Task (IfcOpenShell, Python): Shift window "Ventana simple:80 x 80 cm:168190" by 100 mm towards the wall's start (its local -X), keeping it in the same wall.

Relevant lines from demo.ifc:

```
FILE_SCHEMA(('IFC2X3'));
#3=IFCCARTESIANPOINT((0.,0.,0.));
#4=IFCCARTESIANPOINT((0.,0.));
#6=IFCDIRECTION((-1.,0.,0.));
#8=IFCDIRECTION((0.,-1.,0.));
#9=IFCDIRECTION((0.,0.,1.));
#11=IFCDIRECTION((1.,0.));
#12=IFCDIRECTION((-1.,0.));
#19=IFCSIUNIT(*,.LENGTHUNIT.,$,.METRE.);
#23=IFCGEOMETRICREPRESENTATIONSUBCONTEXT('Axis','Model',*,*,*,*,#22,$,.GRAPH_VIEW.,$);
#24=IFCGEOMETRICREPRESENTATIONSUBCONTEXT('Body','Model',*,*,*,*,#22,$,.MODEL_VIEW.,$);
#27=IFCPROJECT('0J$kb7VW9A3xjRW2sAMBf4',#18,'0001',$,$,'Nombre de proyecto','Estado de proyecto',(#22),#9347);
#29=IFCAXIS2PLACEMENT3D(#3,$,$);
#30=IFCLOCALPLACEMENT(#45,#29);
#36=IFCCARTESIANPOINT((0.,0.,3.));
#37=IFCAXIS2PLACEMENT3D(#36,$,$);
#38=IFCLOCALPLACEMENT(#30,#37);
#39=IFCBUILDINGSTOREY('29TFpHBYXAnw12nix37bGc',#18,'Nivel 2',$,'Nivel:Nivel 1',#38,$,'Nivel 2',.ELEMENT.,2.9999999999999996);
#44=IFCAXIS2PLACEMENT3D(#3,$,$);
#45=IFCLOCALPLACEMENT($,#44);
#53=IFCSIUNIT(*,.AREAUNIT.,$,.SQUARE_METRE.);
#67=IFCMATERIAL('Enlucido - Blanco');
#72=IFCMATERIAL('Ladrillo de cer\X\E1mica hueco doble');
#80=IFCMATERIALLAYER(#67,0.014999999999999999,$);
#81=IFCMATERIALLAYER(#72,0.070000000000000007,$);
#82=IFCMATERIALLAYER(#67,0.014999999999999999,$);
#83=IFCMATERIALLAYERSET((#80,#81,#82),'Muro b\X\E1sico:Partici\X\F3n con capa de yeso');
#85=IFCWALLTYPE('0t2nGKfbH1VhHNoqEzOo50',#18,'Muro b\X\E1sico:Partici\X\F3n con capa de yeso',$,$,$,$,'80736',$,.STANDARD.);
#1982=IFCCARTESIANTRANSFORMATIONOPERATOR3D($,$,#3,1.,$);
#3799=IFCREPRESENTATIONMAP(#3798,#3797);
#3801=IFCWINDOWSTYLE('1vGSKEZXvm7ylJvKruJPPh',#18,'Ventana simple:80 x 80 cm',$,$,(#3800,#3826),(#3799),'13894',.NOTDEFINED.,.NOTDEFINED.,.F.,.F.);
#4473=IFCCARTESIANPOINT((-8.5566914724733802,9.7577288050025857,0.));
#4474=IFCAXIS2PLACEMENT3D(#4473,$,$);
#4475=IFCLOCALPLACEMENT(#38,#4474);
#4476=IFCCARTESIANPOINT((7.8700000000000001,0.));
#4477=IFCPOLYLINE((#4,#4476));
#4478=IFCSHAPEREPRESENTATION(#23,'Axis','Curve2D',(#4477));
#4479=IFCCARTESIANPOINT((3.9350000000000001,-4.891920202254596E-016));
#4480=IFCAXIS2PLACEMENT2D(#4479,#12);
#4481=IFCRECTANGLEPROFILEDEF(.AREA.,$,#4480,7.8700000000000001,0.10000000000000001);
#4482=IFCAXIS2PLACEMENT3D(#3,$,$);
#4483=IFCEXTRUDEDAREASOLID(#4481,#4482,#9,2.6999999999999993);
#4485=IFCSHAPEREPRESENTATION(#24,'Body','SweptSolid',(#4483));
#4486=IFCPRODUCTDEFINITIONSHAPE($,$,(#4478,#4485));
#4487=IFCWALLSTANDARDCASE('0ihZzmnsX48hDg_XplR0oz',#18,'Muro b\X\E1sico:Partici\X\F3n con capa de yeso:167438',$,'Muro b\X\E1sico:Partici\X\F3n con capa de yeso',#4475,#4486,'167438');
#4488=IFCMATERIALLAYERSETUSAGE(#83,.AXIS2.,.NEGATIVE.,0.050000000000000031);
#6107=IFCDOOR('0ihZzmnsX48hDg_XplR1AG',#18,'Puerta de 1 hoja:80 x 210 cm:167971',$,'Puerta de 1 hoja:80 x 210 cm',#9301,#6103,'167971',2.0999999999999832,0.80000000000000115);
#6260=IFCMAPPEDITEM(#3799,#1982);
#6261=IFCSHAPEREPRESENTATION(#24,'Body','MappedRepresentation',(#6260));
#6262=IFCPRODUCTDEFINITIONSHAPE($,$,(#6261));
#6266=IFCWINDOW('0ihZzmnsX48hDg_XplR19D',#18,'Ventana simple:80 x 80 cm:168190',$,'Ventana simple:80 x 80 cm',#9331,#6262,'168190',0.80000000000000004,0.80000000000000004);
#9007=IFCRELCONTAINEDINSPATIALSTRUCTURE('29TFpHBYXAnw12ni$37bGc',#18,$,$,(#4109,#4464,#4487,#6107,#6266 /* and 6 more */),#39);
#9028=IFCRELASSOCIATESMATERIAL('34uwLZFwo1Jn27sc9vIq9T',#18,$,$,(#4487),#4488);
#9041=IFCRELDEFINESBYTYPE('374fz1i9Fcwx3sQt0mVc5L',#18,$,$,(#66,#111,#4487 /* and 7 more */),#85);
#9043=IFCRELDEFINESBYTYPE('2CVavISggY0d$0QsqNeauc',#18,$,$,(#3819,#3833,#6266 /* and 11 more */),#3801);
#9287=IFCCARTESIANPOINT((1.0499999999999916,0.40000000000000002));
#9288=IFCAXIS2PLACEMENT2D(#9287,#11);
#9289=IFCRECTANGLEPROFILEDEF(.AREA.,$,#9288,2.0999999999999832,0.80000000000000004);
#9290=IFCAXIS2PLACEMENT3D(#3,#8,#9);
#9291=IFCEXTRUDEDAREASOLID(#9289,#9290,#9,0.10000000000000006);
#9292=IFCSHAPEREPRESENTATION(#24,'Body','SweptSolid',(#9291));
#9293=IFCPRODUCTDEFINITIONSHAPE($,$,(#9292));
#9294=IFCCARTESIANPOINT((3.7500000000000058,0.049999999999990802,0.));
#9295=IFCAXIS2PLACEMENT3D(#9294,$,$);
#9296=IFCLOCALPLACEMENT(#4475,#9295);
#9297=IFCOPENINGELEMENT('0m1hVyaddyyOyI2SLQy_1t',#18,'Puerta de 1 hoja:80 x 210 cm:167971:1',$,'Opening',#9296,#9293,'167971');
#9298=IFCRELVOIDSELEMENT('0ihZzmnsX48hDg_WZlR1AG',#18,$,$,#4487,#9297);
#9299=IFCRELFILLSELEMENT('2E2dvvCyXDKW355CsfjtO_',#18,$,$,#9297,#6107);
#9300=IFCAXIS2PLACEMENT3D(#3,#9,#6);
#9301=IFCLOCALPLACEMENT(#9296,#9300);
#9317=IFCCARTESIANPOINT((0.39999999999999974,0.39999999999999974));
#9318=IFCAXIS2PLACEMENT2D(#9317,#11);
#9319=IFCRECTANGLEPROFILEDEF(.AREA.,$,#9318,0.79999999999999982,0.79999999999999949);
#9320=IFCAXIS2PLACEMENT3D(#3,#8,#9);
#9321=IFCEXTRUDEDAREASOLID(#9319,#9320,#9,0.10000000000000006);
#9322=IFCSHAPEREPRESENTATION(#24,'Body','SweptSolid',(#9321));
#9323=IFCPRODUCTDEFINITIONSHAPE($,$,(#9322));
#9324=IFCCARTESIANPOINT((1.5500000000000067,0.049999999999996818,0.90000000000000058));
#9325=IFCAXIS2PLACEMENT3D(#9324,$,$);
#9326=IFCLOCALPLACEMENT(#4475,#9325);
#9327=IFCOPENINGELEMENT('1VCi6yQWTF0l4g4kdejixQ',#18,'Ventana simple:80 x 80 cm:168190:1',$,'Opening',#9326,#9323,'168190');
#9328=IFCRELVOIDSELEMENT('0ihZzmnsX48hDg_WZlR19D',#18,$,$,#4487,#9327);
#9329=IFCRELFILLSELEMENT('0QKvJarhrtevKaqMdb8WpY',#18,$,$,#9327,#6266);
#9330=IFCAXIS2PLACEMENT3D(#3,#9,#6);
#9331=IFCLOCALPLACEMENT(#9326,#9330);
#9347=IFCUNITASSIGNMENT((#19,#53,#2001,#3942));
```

```python
import ifcopenshell
import ifcopenshell.api.geometry
import ifcopenshell.util.placement
import ifcopenshell.util.unit

model = ifcopenshell.open("demo.ifc")
unit_scale = ifcopenshell.util.unit.calculate_unit_scale(model)

window = model.by_id(6266)
opening = window.FillsVoids[0].RelatingOpeningElement
wall = opening.VoidsElements[0].RelatingBuildingElement

wall_matrix = ifcopenshell.util.placement.get_local_placement(wall.ObjectPlacement)
shift = wall_matrix[:3, 0] * -0.1 / unit_scale
before = ifcopenshell.util.placement.get_local_placement(window.ObjectPlacement)[:3, 3].copy()

# The window is placed relative to its opening, so it follows when the opening moves.
matrix = ifcopenshell.util.placement.get_local_placement(opening.ObjectPlacement)
matrix[:3, 3] += shift
ifcopenshell.api.geometry.edit_object_placement(
    model, product=opening, matrix=matrix, is_si=False, should_transform_children=True
)

after = ifcopenshell.util.placement.get_local_placement(window.ObjectPlacement)[:3, 3]
print("window moved by", (after - before).round(3) + 0.0)

model.write("demo-out.ifc")
```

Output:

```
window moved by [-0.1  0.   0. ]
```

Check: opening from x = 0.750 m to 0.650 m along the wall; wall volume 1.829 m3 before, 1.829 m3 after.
